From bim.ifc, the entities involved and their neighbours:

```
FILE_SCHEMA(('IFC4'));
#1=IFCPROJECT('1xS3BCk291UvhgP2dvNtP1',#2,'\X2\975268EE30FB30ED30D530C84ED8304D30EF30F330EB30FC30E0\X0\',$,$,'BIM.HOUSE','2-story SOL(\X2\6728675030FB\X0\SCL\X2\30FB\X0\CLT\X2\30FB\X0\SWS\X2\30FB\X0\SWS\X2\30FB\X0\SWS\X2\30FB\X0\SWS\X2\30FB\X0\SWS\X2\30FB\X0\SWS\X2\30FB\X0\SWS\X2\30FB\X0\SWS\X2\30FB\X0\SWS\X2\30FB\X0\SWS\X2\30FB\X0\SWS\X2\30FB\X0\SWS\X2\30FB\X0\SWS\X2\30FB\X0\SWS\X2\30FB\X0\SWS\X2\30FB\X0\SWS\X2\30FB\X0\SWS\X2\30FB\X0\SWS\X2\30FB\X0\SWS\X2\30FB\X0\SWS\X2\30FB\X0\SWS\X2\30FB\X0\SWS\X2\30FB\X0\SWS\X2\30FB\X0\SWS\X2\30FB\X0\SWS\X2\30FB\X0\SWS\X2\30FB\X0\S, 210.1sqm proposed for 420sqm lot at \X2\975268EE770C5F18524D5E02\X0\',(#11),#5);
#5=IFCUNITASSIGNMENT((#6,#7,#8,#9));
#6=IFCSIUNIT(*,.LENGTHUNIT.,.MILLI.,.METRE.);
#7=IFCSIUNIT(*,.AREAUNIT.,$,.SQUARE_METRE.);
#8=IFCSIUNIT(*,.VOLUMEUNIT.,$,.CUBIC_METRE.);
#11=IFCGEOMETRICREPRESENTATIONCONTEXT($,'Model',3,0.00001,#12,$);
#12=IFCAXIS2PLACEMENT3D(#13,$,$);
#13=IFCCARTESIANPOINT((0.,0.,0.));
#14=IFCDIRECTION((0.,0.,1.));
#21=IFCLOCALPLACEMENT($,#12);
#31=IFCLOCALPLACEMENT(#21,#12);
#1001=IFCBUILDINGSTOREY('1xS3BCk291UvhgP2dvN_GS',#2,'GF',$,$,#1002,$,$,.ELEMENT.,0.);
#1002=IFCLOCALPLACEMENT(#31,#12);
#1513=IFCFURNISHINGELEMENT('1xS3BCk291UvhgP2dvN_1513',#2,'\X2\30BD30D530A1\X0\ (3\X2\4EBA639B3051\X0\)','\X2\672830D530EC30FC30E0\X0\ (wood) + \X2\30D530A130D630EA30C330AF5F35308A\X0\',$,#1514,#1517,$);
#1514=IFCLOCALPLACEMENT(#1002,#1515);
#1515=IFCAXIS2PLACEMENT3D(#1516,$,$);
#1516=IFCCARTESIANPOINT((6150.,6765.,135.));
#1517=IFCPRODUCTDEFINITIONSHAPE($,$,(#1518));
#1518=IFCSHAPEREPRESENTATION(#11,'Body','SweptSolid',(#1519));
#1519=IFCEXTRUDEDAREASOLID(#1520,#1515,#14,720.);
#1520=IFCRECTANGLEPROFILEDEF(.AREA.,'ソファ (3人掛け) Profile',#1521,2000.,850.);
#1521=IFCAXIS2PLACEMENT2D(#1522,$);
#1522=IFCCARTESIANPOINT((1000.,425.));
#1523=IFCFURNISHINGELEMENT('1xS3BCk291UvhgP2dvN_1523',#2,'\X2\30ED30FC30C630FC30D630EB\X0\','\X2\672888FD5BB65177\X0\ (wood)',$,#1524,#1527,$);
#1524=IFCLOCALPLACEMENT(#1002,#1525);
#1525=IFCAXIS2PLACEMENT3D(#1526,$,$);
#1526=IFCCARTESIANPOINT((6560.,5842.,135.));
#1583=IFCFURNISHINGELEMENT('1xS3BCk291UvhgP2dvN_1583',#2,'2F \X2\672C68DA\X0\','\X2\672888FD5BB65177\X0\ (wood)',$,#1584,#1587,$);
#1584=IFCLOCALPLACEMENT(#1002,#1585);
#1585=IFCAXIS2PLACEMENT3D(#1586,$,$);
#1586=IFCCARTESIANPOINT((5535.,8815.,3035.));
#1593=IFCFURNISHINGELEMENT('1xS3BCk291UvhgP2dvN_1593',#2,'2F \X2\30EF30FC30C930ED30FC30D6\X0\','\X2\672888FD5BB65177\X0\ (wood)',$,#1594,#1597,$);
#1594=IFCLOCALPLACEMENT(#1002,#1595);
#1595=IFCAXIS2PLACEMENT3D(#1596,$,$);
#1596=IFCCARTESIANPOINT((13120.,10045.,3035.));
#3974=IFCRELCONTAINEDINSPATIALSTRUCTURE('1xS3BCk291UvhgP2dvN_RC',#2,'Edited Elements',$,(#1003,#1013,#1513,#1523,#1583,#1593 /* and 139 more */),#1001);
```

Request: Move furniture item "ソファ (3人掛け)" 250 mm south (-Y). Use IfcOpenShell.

```python
import ifcopenshell
import ifcopenshell.api.geometry
import ifcopenshell.util.placement

model = ifcopenshell.open("bim.ifc")

item = model.by_guid("1xS3BCk291UvhgP2dvN_1513")
matrix = ifcopenshell.util.placement.get_local_placement(item.ObjectPlacement)
matrix[1, 3] -= 250.0
ifcopenshell.api.geometry.edit_object_placement(model, product=item, matrix=matrix, is_si=False)

print(ifcopenshell.util.placement.get_local_placement(item.ObjectPlacement).round(3) + 0.0)

model.write("bim_updated.ifc")
```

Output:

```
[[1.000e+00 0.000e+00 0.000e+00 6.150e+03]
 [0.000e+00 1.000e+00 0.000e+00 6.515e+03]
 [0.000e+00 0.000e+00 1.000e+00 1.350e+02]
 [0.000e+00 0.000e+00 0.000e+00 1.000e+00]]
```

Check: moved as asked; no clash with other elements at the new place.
